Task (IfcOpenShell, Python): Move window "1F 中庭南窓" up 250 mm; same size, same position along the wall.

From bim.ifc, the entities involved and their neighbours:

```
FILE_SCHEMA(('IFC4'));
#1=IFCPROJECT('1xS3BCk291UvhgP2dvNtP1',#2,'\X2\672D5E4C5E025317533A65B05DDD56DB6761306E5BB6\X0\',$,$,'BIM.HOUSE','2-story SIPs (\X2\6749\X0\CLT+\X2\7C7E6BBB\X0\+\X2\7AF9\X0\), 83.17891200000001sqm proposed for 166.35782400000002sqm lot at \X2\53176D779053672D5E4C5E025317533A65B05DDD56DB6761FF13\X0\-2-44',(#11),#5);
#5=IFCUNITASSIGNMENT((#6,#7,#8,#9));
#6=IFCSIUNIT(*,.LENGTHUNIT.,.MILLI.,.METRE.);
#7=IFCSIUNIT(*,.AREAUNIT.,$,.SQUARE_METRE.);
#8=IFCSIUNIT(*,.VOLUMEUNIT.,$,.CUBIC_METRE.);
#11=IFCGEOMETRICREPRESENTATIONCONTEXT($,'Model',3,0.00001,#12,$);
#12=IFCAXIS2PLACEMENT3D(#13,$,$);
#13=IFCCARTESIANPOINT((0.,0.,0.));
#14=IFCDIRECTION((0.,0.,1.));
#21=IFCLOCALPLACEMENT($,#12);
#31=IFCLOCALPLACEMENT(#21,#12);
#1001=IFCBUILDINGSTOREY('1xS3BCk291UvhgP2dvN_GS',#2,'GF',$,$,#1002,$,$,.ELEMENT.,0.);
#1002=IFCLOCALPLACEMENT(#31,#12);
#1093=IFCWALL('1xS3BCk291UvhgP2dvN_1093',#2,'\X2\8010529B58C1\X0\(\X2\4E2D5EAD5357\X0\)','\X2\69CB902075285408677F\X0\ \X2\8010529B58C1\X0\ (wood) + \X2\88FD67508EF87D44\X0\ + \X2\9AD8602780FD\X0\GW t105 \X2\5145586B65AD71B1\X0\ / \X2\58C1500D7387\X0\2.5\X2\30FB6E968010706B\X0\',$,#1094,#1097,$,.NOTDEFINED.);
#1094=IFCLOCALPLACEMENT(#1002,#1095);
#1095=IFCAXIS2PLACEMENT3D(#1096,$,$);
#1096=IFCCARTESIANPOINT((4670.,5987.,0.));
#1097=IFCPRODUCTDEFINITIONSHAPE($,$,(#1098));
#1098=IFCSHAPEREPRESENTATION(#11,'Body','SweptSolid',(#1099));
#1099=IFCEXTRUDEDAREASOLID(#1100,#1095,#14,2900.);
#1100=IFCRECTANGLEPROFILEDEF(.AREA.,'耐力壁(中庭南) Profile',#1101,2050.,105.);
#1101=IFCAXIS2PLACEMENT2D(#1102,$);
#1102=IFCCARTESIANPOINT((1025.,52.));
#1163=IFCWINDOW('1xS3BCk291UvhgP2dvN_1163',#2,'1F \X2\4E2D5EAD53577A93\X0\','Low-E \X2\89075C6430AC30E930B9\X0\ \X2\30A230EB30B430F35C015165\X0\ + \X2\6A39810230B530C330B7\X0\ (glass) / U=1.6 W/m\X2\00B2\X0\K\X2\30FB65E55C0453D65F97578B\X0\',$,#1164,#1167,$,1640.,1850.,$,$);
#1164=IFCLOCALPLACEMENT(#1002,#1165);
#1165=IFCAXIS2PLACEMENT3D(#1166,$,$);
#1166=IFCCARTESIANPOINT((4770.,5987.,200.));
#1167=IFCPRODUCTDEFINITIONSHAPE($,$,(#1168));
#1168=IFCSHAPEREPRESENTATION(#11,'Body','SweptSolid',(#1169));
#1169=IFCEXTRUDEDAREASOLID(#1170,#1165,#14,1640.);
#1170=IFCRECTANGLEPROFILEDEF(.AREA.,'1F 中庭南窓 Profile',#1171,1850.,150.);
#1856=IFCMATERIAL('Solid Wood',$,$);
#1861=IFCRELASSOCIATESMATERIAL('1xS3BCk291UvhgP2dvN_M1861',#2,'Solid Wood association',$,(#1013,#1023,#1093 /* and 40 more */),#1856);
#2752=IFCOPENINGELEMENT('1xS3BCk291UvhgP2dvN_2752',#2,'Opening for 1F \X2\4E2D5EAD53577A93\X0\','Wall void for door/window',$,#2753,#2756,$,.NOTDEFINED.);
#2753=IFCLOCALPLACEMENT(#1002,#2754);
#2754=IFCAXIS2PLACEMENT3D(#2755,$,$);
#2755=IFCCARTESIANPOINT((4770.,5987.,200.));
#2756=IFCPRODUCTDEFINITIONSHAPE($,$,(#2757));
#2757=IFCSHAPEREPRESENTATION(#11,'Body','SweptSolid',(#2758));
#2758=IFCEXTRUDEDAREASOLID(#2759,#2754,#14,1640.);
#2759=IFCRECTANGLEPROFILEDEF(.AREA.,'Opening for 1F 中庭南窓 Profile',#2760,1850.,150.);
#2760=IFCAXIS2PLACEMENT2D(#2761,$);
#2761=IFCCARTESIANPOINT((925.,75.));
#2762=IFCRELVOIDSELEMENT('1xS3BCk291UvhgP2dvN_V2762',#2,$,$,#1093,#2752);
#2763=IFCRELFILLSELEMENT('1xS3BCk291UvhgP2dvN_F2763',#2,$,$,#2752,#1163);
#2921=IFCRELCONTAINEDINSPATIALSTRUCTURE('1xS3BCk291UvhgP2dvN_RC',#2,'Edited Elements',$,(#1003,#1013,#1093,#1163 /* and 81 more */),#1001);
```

```python
import numpy as np
import ifcopenshell
import ifcopenshell.api.geometry
import ifcopenshell.util.placement
import ifcopenshell.util.unit

model = ifcopenshell.open("bim.ifc")
unit_scale = ifcopenshell.util.unit.calculate_unit_scale(model)

window = model.by_id(1163)
opening = window.FillsVoids[0].RelatingOpeningElement
dz = 0.25 / unit_scale

shift = np.array([0.0, 0.0, dz])
# The window is not placed relative to its opening, so move both.
for product in (opening, window):
    matrix = ifcopenshell.util.placement.get_local_placement(product.ObjectPlacement)
    matrix[:3, 3] += shift
    ifcopenshell.api.geometry.edit_object_placement(model, product=product, matrix=matrix, is_si=False)

print(f"moved by {dz * unit_scale:+.3f} m")

model.write("bim_updated.ifc")
```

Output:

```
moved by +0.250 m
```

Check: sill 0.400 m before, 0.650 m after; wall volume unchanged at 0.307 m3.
